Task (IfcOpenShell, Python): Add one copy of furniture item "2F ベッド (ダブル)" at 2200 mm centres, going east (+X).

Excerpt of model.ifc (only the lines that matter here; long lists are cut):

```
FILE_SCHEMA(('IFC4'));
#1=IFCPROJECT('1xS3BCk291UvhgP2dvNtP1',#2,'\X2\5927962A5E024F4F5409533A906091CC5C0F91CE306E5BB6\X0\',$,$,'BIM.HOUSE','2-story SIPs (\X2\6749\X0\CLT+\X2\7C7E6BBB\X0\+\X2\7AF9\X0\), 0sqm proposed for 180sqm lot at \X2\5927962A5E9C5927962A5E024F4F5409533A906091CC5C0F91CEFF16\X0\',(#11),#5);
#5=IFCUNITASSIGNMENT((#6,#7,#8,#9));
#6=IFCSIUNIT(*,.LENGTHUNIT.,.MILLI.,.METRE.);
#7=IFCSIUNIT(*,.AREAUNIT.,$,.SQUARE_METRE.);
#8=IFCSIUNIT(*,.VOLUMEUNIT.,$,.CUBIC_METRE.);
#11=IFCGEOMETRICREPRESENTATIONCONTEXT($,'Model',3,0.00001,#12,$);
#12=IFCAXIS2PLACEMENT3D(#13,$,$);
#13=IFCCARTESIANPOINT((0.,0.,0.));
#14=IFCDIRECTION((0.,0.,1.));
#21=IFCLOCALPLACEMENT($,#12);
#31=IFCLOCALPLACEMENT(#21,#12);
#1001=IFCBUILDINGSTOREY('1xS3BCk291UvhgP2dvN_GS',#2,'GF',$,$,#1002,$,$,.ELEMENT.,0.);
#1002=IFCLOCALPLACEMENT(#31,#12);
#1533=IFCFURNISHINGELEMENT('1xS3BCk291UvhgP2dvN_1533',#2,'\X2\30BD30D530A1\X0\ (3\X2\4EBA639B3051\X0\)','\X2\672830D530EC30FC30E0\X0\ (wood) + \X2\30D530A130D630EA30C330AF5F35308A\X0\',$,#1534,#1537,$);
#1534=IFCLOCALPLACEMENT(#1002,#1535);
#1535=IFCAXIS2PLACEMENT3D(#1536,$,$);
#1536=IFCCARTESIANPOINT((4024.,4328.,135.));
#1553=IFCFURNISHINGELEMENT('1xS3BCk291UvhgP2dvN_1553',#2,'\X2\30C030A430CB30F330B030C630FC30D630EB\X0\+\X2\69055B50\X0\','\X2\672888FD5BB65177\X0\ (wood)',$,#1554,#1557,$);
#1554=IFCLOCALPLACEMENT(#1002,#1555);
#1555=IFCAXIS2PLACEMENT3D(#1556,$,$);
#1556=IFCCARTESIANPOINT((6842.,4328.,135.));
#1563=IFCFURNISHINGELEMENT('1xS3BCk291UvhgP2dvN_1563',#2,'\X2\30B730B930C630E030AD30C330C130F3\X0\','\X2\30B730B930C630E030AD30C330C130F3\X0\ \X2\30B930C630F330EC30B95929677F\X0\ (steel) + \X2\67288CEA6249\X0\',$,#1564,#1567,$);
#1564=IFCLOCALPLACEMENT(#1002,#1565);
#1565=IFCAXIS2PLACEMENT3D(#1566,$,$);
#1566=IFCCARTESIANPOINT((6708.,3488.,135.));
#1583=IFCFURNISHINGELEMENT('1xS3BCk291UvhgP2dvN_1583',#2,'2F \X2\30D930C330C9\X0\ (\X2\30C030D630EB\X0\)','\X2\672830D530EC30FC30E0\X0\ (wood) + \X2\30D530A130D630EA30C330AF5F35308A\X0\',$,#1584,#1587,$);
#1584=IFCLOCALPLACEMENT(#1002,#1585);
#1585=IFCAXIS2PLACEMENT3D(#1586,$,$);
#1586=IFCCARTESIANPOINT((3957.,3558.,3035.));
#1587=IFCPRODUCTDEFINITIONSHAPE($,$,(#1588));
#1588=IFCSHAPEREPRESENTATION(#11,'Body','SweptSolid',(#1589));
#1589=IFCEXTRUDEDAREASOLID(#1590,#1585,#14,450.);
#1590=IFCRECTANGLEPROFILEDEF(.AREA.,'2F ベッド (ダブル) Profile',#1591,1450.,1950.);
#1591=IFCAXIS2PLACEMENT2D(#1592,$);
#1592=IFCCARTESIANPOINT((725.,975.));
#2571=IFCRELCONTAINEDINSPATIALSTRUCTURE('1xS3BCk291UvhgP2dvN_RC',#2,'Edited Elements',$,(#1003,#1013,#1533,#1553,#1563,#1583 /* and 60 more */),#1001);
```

```python
import numpy as np
import ifcopenshell
import ifcopenshell.api.geometry
import ifcopenshell.api.root
import ifcopenshell.util.element
import ifcopenshell.util.placement
import ifcopenshell.util.unit

model = ifcopenshell.open("model.ifc")
unit_scale = ifcopenshell.util.unit.calculate_unit_scale(model)


def reuse_history(source, copy):
    """copy_class also copies each property set's owner history, people and application; keep the originals."""
    for rel in copy.IsDefinedBy:
        if rel.is_a("IfcRelDefinesByProperties") and (history := rel.RelatingPropertyDefinition.OwnerHistory):
            rel.RelatingPropertyDefinition.OwnerHistory = source.OwnerHistory
            ifcopenshell.util.element.remove_deep2(model, history)


source = model.by_guid("1xS3BCk291UvhgP2dvN_1583")
base = ifcopenshell.util.placement.get_local_placement(source.ObjectPlacement)
step = np.array([1.0, 0.0, 0.0]) * 2.2 / unit_scale

for i in range(1, 2):
    copy = ifcopenshell.api.root.copy_class(model, product=source)
    copy.Representation = ifcopenshell.util.element.copy_deep(
        model, source.Representation, exclude=["IfcGeometricRepresentationContext", "IfcRepresentationMap"]
    )
    reuse_history(source, copy)
    matrix = base.copy()
    matrix[:3, 3] += i * step
    print("added at", matrix[:3, 3].round(3) + 0.0)
    ifcopenshell.api.geometry.edit_object_placement(model, product=copy, matrix=matrix, is_si=False)

model.write("model_updated.ifc")
```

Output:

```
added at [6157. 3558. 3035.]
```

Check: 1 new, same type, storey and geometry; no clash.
